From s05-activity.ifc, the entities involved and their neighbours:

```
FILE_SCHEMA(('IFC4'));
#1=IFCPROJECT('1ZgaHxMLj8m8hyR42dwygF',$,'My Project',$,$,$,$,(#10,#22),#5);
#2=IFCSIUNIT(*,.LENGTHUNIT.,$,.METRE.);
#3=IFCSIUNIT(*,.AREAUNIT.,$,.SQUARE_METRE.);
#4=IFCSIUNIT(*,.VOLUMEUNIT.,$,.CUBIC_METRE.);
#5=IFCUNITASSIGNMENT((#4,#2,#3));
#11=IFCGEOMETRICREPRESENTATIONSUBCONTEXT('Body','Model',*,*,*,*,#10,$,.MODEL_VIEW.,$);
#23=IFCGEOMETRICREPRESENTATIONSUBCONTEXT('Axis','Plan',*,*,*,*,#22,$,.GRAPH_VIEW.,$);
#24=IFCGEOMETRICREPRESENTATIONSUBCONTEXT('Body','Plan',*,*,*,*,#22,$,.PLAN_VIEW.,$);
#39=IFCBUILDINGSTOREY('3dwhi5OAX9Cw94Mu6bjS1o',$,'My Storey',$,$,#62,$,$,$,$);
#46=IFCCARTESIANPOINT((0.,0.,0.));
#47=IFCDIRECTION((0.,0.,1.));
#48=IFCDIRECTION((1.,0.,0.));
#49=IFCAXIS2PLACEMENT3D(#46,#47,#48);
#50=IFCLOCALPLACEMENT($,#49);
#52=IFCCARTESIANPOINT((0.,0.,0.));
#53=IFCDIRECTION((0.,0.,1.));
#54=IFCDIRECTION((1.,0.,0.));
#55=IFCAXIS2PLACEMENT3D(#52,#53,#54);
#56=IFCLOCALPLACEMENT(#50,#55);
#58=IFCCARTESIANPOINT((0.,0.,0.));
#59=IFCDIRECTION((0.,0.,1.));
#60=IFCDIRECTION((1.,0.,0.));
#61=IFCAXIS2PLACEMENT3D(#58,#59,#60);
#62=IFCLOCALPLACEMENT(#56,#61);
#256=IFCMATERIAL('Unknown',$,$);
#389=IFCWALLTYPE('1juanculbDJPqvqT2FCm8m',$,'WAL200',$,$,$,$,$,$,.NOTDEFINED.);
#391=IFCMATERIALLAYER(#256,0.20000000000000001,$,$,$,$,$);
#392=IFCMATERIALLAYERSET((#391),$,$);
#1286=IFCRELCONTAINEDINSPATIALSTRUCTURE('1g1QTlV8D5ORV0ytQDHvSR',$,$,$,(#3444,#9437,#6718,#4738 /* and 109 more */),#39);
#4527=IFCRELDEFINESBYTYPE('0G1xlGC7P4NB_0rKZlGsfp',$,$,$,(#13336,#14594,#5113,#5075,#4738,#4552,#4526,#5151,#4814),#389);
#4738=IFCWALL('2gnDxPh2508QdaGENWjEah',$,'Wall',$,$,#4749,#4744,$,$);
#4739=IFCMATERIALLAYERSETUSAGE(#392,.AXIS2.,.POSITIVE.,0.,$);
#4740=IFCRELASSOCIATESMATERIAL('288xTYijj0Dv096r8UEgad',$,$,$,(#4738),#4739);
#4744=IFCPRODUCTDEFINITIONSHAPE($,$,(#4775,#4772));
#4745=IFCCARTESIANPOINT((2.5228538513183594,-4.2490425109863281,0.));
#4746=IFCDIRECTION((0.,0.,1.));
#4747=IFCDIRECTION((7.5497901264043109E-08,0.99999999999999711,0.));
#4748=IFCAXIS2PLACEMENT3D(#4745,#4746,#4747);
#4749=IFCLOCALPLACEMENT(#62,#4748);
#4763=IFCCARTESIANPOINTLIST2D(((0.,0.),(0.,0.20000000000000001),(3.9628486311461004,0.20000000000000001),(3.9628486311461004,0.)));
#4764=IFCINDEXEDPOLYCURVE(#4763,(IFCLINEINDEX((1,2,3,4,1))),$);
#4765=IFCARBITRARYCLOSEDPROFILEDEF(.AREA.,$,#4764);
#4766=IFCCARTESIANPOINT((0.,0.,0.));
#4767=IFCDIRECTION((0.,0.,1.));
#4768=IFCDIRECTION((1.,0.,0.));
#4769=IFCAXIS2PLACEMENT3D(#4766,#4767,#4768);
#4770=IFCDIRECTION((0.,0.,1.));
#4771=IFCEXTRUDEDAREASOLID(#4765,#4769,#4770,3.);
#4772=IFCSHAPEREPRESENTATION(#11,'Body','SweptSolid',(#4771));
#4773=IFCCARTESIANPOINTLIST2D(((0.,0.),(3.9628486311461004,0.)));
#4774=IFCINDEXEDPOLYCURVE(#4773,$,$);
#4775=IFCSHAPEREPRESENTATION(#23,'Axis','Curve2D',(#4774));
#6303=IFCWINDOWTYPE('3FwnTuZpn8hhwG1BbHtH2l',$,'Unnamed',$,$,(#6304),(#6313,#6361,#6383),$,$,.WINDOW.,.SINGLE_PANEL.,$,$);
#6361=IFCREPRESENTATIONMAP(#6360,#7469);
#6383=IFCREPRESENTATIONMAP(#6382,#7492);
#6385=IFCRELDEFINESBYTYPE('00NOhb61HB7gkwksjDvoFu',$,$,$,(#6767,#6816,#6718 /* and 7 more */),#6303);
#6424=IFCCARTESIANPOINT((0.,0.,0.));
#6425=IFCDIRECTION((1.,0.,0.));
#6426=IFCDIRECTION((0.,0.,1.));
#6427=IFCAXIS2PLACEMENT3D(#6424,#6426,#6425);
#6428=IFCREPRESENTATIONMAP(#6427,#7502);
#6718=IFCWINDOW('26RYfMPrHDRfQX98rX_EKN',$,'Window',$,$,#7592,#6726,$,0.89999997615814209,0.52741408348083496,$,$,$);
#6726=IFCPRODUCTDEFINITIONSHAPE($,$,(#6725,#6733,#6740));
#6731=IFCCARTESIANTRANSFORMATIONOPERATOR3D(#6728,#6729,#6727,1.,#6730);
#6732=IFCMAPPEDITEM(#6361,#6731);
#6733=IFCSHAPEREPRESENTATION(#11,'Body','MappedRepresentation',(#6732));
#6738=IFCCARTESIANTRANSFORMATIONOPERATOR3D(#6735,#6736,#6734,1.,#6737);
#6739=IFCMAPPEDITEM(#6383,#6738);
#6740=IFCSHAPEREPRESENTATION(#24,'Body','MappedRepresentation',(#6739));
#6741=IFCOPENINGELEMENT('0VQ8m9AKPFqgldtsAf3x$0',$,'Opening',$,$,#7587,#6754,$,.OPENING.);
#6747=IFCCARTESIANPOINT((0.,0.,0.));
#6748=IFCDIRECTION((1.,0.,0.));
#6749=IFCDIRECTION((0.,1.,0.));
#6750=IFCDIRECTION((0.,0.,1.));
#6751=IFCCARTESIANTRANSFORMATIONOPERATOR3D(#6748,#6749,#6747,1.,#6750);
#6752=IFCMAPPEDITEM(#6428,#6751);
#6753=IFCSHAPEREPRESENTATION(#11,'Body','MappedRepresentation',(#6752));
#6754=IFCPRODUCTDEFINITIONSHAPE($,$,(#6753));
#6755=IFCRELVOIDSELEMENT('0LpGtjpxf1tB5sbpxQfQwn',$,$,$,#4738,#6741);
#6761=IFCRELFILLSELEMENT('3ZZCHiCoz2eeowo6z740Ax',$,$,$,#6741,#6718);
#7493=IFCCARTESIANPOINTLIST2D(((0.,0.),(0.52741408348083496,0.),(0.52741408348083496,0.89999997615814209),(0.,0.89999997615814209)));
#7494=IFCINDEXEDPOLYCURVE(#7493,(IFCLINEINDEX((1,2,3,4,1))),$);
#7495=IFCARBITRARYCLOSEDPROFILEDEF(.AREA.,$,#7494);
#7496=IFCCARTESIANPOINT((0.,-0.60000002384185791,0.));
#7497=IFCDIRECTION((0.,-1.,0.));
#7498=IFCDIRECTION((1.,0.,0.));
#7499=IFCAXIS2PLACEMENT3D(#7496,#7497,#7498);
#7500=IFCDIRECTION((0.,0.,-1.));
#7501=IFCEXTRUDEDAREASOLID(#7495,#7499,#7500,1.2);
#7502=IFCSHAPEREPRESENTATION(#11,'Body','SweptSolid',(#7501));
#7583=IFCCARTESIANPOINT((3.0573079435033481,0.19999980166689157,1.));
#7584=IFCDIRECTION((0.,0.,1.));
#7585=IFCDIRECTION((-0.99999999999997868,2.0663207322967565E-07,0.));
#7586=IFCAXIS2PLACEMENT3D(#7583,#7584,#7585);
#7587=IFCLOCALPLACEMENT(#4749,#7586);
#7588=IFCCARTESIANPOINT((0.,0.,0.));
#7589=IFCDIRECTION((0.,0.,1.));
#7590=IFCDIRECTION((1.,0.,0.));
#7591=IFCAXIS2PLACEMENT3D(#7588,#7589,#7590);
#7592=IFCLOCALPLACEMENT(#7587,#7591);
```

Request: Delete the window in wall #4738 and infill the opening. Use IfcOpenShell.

```python
import ifcopenshell
import ifcopenshell.api.feature
import ifcopenshell.api.root
import ifcopenshell.geom
import ifcopenshell.util.shape

model = ifcopenshell.open("s05-activity.ifc")
settings = ifcopenshell.geom.settings()


def volume(element):
    """Net volume in cubic metres, openings subtracted."""
    shape = ifcopenshell.geom.create_shape(settings, element)
    return ifcopenshell.util.shape.get_volume(shape.geometry)


window = model.by_guid("26RYfMPrHDRfQX98rX_EKN")
opening = window.FillsVoids[0].RelatingOpeningElement
wall = opening.VoidsElements[0].RelatingBuildingElement
before = volume(wall)

ifcopenshell.api.root.remove_product(model, product=window)
ifcopenshell.api.feature.remove_feature(model, feature=opening)

after = volume(wall)

print(f"wall volume {before:.3f} -> {after:.3f} m3")

model.write("s05-activity-out.ifc")
```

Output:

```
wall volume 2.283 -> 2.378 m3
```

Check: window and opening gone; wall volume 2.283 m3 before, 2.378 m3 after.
